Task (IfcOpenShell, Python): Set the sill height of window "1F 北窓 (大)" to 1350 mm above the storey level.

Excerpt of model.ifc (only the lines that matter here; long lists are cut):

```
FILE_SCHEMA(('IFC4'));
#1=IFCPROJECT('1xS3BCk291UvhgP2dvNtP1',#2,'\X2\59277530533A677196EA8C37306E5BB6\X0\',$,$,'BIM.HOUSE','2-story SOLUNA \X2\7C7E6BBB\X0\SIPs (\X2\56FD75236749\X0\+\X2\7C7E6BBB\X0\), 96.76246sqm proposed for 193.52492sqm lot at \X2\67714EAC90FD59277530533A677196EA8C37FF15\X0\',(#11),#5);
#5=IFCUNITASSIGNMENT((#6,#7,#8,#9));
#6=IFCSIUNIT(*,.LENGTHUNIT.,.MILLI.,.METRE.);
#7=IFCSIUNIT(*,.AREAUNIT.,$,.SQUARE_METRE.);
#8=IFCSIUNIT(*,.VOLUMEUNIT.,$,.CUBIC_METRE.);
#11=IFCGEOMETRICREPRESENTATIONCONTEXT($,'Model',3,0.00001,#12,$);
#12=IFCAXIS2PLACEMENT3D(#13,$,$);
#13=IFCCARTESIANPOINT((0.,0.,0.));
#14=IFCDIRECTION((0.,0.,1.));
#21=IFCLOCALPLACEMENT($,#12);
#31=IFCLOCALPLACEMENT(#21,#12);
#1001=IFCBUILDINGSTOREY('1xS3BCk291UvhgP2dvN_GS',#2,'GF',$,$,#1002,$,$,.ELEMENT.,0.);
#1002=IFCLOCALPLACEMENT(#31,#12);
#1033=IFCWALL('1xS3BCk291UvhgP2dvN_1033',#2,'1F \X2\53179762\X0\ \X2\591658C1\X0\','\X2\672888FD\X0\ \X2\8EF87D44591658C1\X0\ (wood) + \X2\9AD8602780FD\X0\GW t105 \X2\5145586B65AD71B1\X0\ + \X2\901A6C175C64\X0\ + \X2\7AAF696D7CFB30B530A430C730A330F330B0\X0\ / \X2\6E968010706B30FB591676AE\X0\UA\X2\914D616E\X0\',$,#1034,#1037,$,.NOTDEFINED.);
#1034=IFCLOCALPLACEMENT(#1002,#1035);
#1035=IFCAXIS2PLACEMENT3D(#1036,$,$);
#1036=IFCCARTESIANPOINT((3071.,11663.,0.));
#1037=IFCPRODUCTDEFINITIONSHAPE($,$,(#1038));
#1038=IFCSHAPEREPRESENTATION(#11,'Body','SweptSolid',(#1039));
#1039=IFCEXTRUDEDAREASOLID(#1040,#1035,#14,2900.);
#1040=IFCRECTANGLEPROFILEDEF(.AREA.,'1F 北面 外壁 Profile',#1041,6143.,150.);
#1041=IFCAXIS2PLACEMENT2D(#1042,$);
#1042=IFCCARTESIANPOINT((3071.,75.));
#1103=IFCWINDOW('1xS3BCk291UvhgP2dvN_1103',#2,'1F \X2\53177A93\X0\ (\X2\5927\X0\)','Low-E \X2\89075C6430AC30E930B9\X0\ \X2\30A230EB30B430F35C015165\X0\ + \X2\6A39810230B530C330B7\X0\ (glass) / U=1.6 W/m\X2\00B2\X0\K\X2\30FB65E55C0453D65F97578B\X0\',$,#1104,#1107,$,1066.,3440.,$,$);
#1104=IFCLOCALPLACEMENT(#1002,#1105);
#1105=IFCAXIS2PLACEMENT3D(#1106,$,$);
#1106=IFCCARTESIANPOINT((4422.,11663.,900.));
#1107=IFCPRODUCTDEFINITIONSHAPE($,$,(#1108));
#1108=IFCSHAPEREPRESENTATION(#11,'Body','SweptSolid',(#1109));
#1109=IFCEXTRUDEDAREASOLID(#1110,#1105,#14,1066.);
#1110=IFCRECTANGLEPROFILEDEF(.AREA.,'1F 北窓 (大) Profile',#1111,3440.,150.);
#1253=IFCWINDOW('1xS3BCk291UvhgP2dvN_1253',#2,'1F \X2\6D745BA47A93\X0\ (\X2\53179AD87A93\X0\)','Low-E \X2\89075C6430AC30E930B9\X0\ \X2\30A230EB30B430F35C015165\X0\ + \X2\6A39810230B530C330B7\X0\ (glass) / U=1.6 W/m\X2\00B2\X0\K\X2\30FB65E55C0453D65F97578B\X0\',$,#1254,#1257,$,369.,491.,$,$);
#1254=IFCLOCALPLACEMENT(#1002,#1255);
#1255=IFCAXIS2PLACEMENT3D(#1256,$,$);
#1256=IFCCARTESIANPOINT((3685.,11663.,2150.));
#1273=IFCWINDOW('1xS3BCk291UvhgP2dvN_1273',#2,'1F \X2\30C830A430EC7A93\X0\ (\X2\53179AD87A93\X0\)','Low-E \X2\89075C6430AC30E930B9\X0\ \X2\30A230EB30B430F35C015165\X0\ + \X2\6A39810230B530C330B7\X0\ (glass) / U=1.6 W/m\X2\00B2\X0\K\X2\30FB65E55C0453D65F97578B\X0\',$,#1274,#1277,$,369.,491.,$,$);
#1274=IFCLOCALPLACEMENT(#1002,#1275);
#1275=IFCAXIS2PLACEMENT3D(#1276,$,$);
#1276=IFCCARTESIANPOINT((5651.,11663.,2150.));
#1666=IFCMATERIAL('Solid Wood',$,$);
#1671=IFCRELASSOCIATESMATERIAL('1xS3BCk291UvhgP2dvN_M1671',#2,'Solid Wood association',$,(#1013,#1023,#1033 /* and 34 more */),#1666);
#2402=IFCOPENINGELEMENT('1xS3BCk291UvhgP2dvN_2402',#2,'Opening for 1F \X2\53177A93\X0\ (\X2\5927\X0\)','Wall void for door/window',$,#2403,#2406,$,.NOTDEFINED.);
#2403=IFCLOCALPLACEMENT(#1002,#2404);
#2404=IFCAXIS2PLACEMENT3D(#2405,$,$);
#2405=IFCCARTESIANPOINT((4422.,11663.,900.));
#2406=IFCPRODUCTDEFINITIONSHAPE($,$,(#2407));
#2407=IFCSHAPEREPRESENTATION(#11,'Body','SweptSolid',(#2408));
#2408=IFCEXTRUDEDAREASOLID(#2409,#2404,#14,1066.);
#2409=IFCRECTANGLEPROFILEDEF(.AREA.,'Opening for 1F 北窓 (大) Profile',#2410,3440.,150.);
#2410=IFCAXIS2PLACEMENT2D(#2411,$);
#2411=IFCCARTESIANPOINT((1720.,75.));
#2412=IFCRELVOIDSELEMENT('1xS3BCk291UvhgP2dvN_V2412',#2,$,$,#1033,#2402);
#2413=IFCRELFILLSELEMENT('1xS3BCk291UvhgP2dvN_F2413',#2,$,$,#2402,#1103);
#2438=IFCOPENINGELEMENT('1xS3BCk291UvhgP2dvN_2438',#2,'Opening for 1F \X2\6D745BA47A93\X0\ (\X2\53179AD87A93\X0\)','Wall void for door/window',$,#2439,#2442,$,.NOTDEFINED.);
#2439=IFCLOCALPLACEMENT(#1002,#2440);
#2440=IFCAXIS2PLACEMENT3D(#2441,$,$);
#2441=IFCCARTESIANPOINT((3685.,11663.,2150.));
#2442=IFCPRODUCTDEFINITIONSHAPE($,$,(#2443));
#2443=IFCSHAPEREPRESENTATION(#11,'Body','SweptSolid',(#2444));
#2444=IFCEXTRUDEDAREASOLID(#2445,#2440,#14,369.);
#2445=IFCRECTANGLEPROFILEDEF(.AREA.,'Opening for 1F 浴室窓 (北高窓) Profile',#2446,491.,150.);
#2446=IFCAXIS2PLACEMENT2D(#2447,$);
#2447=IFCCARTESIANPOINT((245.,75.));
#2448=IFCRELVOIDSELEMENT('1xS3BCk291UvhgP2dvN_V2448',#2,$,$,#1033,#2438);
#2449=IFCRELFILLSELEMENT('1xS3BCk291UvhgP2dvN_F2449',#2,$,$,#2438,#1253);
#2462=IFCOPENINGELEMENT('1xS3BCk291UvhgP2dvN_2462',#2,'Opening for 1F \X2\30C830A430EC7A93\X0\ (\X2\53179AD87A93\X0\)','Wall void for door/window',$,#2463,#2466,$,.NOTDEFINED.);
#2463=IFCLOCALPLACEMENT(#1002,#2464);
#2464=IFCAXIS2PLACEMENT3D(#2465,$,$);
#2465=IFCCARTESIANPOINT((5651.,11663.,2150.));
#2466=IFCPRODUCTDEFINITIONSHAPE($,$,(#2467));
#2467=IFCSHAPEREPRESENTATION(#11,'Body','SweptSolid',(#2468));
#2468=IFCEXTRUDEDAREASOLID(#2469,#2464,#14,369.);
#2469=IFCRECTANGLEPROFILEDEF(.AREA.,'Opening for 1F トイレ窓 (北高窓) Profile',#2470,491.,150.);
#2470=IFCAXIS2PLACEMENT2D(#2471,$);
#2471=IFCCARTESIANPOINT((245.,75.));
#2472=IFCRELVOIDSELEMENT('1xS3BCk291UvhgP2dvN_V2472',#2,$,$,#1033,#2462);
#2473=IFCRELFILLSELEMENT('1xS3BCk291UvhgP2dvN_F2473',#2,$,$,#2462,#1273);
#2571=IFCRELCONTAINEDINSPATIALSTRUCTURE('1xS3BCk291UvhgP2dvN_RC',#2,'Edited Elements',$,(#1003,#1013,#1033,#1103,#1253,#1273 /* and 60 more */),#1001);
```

```python
import numpy as np
import ifcopenshell
import ifcopenshell.api.geometry
import ifcopenshell.geom
import ifcopenshell.util.element
import ifcopenshell.util.placement
import ifcopenshell.util.shape
import ifcopenshell.util.unit

model = ifcopenshell.open("model.ifc")
unit_scale = ifcopenshell.util.unit.calculate_unit_scale(model)

window = model.by_guid("1xS3BCk291UvhgP2dvN_1103")
opening = window.FillsVoids[0].RelatingOpeningElement
storey = ifcopenshell.util.element.get_container(window, ifc_class="IfcBuildingStorey")
level = ifcopenshell.util.placement.get_local_placement(storey.ObjectPlacement)[2, 3]

# The opening's origin need not be at the sill, so measure its lowest point.
shape = ifcopenshell.geom.create_shape(ifcopenshell.geom.settings(), opening)
bottom = ifcopenshell.util.shape.get_shape_bottom_elevation(shape, shape.geometry) / unit_scale
dz = level + 1350.0 - bottom

shift = np.array([0.0, 0.0, dz])
# The window is not placed relative to its opening, so move both.
for product in (opening, window):
    matrix = ifcopenshell.util.placement.get_local_placement(product.ObjectPlacement)
    matrix[:3, 3] += shift
    ifcopenshell.api.geometry.edit_object_placement(model, product=product, matrix=matrix, is_si=False)

print(f"moved by {dz * unit_scale:+.3f} m")

model.write("model_v2.ifc")
```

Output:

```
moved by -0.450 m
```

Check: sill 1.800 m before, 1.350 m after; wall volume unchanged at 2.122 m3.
